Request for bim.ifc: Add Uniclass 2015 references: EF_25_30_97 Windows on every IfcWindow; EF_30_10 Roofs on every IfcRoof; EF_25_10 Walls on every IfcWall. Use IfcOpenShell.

First a look at what the model holds.

```python
import ifcopenshell

model = ifcopenshell.open("bim.ifc")
print(model.schema)
print("classifications:", [c.Name for c in model.by_type("IfcClassification")])
for ifc_class in ("IfcDoor", "IfcRoof", "IfcStair", "IfcWall", "IfcWindow"):
    print(ifc_class, len(model.by_type(ifc_class)))
```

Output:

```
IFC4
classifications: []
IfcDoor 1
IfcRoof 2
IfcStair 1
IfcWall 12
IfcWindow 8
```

```python
import ifcopenshell
import ifcopenshell.api.classification

model = ifcopenshell.open("bim.ifc")

system = ifcopenshell.api.classification.add_classification(model, classification="Uniclass 2015")

codes = {
    "IfcWindow": ("EF_25_30_97", "Windows"),
    "IfcRoof": ("EF_30_10", "Roofs"),
    "IfcWall": ("EF_25_10", "Walls"),
}
for ifc_class, (code, name) in codes.items():
    products = model.by_type(ifc_class)
    ifcopenshell.api.classification.add_reference(
        model, products=products, classification=system, identification=code, name=name
    )
    print(code, len(products))

model.write("bim_edited.ifc")
```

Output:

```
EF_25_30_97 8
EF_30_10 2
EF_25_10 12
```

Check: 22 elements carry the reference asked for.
